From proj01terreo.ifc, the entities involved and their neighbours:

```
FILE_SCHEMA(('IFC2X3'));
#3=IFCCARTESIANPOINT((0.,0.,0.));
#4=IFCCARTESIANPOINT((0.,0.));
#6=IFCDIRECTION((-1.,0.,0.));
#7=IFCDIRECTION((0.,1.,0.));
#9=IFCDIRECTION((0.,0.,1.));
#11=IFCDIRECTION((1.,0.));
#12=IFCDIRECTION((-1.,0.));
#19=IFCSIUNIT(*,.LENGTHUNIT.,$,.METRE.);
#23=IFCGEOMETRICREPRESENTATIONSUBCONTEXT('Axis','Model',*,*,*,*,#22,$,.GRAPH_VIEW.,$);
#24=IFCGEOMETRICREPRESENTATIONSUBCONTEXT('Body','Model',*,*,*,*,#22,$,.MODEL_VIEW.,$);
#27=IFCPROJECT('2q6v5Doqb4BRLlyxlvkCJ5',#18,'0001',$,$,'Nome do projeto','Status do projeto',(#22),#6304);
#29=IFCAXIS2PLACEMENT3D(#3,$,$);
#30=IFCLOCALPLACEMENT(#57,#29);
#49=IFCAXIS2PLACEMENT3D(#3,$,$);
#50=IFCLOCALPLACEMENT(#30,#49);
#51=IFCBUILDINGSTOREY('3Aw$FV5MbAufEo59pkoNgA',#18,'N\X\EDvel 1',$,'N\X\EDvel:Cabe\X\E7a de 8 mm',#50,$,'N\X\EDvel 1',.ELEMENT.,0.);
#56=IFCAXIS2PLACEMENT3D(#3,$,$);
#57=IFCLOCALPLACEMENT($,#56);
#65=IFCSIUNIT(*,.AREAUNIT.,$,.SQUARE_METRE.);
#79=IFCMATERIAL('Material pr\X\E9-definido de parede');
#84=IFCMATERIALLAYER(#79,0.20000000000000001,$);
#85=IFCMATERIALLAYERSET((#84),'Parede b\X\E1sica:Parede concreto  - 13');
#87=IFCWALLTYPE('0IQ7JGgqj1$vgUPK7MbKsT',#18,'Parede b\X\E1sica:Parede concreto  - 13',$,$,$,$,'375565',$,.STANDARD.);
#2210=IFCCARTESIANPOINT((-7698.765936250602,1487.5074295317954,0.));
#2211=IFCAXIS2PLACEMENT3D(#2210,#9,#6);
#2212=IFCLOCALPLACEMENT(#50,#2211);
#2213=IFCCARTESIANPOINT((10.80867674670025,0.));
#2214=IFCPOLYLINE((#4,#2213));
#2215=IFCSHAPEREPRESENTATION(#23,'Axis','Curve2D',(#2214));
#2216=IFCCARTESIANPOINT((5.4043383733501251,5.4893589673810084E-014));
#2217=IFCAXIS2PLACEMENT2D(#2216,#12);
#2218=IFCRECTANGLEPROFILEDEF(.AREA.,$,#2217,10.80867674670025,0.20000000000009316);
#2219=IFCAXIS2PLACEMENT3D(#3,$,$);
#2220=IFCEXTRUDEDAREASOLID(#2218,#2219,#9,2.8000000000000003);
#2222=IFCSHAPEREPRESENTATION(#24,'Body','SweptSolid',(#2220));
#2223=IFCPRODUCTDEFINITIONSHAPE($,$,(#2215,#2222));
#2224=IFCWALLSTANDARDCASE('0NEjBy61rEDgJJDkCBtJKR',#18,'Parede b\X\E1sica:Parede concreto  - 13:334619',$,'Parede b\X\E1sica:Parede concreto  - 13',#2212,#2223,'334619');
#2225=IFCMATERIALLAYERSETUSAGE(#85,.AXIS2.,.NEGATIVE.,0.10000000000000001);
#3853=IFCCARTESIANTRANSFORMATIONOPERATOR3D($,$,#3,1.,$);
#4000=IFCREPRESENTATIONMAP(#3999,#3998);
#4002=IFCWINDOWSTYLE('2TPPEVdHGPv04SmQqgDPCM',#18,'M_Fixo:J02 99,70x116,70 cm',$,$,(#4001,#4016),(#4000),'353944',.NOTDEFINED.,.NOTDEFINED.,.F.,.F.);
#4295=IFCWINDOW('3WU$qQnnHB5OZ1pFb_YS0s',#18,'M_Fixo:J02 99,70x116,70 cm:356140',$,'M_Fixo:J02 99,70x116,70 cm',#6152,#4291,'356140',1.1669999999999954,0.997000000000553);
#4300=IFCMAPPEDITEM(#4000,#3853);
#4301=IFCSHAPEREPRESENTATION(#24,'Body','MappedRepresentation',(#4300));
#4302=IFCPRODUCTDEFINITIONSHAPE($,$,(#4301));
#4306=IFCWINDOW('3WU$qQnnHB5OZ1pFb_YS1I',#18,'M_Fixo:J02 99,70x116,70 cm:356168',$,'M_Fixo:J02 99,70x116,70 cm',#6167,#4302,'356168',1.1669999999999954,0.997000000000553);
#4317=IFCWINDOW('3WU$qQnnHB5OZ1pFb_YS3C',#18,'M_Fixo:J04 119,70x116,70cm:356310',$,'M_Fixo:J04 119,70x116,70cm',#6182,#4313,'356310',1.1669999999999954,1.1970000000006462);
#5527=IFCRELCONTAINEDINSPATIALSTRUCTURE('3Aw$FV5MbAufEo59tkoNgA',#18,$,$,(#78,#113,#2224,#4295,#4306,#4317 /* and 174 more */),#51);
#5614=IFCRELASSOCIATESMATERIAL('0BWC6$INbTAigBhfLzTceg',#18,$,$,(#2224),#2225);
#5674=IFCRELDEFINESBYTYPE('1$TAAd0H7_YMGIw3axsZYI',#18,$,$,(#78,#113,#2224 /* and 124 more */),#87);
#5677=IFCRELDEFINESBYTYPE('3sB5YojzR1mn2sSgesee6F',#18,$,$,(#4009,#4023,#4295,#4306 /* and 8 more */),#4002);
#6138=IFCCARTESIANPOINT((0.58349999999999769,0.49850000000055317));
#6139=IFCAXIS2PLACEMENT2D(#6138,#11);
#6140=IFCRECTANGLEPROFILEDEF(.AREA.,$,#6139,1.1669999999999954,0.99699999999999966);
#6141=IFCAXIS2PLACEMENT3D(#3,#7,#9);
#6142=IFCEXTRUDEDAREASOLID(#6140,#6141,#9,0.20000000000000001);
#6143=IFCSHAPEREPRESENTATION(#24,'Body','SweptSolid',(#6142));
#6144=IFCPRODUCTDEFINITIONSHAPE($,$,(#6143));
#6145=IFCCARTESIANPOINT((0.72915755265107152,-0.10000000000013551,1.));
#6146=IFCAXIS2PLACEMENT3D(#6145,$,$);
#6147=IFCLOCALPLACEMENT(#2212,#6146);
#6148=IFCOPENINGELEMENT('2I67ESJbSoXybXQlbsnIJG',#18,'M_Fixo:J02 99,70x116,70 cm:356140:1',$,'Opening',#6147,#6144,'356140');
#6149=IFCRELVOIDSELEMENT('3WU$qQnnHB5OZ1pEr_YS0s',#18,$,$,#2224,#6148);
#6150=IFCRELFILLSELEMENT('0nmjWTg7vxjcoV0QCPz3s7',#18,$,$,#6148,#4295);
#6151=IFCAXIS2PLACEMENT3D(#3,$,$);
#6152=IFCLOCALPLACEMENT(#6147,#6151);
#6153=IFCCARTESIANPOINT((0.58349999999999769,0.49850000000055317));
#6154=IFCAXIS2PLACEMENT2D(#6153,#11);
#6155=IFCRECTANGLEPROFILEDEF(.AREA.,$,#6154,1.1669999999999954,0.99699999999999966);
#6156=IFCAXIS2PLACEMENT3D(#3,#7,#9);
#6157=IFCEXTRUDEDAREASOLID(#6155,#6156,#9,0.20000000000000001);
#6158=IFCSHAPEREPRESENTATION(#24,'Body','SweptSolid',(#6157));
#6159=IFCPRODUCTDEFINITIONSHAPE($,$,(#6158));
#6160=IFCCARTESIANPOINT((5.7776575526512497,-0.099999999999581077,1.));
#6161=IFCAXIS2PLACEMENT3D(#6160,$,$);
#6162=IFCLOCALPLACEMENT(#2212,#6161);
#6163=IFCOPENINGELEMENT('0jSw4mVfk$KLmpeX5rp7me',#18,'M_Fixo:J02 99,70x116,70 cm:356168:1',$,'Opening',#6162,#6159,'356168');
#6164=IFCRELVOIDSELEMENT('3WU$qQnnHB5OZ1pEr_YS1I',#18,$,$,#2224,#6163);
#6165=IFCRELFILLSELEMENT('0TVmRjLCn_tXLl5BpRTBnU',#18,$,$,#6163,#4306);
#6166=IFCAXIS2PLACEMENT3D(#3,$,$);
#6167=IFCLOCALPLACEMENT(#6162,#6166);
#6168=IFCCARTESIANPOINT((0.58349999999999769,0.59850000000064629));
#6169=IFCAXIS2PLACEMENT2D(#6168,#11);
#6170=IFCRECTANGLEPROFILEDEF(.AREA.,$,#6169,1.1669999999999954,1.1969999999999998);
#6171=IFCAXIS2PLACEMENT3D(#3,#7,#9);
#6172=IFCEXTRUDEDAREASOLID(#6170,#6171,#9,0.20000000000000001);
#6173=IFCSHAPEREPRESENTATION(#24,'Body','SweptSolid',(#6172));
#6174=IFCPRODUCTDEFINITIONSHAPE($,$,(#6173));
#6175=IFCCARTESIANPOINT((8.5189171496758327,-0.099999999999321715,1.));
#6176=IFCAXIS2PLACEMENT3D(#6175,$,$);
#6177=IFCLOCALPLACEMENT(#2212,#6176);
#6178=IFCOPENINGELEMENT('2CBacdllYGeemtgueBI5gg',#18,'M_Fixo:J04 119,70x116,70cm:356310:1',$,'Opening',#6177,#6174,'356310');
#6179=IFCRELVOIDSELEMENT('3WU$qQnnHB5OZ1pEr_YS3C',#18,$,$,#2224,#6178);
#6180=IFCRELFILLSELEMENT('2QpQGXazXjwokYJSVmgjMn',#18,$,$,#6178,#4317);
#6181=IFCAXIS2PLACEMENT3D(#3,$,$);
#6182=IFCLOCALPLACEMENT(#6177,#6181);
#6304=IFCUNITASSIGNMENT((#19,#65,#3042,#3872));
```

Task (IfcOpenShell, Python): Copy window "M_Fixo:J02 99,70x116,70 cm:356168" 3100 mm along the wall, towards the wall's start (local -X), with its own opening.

```python
import ifcopenshell
import ifcopenshell.api.feature
import ifcopenshell.api.geometry
import ifcopenshell.api.root
import ifcopenshell.geom
import ifcopenshell.util.element
import ifcopenshell.util.placement
import ifcopenshell.util.shape
import ifcopenshell.util.unit

model = ifcopenshell.open("proj01terreo.ifc")
unit_scale = ifcopenshell.util.unit.calculate_unit_scale(model)
settings = ifcopenshell.geom.settings()


def volume(element):
    """Net volume in cubic metres, openings subtracted."""
    shape = ifcopenshell.geom.create_shape(settings, element)
    return ifcopenshell.util.shape.get_volume(shape.geometry)


def reuse_history(source, copy):
    """copy_class also copies each property set's owner history, people and application; keep the originals."""
    for rel in copy.IsDefinedBy:
        if rel.is_a("IfcRelDefinesByProperties") and (history := rel.RelatingPropertyDefinition.OwnerHistory):
            rel.RelatingPropertyDefinition.OwnerHistory = source.OwnerHistory
            ifcopenshell.util.element.remove_deep2(model, history)


window = model.by_id(4306)
opening = window.FillsVoids[0].RelatingOpeningElement
wall = opening.VoidsElements[0].RelatingBuildingElement
before = volume(wall)
shift = ifcopenshell.util.placement.get_local_placement(wall.ObjectPlacement)[:3, 0] * -3.1 / unit_scale

# copy_class copies the void relationship, type, container and properties, but no geometry.
new_opening = ifcopenshell.api.root.copy_class(model, product=opening)
new_opening.Representation = ifcopenshell.util.element.copy_deep(
    model, opening.Representation, exclude=["IfcGeometricRepresentationContext", "IfcRepresentationMap"]
)
new_opening.Name = "M_Fixo:J02 99,70x116,70 cm"
new_opening.Tag = None
new_window = ifcopenshell.api.root.copy_class(model, product=window)
new_window.Representation = ifcopenshell.util.element.copy_deep(
    model, window.Representation, exclude=["IfcGeometricRepresentationContext", "IfcRepresentationMap"]
)
new_window.Name = "M_Fixo:J02 99,70x116,70 cm"
new_window.Tag = None
reuse_history(window, new_window)
fills = ifcopenshell.api.feature.add_filling(model, opening=new_opening, element=new_window)
fills.OwnerHistory = new_window.OwnerHistory  # required in IFC2X3

for old, new in ((opening, new_opening), (window, new_window)):
    matrix = ifcopenshell.util.placement.get_local_placement(old.ObjectPlacement)
    matrix[:3, 3] += shift
    ifcopenshell.api.geometry.edit_object_placement(model, product=new, matrix=matrix, is_si=False)

after = volume(wall)

print(f"wall volume {before:.3f} -> {after:.3f} m3")

model.write("proj01terreo_updated.ifc")
```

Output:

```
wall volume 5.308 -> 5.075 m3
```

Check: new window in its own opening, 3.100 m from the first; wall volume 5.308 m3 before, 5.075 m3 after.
